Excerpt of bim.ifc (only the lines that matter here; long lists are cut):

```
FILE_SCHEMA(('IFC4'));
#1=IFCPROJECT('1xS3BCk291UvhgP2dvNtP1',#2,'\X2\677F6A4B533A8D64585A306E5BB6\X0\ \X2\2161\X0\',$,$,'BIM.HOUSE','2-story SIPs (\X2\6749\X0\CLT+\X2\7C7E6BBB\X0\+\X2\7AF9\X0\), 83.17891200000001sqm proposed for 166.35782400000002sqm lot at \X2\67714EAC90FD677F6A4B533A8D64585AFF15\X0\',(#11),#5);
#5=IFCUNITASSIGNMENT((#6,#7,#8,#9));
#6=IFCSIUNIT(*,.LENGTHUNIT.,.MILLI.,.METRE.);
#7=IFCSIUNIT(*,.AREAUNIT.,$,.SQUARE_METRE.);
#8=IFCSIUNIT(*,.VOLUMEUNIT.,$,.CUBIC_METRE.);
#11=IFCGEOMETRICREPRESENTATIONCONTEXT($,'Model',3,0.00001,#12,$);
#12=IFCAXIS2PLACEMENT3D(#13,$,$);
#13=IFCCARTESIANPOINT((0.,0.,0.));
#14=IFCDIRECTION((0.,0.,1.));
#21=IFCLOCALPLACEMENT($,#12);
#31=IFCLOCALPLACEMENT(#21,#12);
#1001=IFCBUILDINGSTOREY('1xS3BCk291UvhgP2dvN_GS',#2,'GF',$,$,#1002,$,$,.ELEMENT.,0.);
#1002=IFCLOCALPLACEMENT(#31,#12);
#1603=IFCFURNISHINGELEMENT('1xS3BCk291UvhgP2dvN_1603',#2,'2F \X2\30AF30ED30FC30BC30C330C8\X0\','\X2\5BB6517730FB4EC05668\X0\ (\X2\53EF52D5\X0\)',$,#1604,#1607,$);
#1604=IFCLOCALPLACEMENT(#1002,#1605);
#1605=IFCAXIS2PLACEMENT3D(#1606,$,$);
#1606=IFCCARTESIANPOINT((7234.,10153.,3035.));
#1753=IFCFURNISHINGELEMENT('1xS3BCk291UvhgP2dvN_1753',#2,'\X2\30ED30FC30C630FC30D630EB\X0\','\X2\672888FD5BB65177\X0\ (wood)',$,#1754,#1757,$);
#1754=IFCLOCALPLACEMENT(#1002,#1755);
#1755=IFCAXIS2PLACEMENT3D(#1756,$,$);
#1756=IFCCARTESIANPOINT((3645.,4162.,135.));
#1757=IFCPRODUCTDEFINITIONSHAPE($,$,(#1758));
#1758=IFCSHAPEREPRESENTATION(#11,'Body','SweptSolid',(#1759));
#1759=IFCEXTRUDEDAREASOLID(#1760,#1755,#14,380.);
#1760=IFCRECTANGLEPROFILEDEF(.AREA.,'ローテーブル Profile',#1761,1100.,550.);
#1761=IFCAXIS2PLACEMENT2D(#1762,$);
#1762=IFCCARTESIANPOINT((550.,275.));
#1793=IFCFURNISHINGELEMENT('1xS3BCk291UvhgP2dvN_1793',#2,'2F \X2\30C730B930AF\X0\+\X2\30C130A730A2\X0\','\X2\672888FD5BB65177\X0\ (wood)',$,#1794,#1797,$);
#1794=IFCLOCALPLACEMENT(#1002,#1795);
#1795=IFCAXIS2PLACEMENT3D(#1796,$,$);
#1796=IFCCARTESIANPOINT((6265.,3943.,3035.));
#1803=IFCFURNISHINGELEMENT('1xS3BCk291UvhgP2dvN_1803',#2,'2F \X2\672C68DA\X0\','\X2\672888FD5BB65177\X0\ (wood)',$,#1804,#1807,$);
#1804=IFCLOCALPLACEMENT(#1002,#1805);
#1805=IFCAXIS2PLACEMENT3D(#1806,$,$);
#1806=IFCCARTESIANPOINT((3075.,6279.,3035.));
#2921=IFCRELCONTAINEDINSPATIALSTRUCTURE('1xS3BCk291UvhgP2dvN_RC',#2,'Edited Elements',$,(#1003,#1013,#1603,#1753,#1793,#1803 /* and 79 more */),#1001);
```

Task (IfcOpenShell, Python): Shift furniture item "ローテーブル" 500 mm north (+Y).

```python
import ifcopenshell
import ifcopenshell.api.geometry
import ifcopenshell.util.placement

model = ifcopenshell.open("bim.ifc")

item = model.by_guid("1xS3BCk291UvhgP2dvN_1753")
matrix = ifcopenshell.util.placement.get_local_placement(item.ObjectPlacement)
matrix[1, 3] += 500.0
ifcopenshell.api.geometry.edit_object_placement(model, product=item, matrix=matrix, is_si=False)

print(ifcopenshell.util.placement.get_local_placement(item.ObjectPlacement).round(3) + 0.0)

model.write("bim_v2.ifc")
```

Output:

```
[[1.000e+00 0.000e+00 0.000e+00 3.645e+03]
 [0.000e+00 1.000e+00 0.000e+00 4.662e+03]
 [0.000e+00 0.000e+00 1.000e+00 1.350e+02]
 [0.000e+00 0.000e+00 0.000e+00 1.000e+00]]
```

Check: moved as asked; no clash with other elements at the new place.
